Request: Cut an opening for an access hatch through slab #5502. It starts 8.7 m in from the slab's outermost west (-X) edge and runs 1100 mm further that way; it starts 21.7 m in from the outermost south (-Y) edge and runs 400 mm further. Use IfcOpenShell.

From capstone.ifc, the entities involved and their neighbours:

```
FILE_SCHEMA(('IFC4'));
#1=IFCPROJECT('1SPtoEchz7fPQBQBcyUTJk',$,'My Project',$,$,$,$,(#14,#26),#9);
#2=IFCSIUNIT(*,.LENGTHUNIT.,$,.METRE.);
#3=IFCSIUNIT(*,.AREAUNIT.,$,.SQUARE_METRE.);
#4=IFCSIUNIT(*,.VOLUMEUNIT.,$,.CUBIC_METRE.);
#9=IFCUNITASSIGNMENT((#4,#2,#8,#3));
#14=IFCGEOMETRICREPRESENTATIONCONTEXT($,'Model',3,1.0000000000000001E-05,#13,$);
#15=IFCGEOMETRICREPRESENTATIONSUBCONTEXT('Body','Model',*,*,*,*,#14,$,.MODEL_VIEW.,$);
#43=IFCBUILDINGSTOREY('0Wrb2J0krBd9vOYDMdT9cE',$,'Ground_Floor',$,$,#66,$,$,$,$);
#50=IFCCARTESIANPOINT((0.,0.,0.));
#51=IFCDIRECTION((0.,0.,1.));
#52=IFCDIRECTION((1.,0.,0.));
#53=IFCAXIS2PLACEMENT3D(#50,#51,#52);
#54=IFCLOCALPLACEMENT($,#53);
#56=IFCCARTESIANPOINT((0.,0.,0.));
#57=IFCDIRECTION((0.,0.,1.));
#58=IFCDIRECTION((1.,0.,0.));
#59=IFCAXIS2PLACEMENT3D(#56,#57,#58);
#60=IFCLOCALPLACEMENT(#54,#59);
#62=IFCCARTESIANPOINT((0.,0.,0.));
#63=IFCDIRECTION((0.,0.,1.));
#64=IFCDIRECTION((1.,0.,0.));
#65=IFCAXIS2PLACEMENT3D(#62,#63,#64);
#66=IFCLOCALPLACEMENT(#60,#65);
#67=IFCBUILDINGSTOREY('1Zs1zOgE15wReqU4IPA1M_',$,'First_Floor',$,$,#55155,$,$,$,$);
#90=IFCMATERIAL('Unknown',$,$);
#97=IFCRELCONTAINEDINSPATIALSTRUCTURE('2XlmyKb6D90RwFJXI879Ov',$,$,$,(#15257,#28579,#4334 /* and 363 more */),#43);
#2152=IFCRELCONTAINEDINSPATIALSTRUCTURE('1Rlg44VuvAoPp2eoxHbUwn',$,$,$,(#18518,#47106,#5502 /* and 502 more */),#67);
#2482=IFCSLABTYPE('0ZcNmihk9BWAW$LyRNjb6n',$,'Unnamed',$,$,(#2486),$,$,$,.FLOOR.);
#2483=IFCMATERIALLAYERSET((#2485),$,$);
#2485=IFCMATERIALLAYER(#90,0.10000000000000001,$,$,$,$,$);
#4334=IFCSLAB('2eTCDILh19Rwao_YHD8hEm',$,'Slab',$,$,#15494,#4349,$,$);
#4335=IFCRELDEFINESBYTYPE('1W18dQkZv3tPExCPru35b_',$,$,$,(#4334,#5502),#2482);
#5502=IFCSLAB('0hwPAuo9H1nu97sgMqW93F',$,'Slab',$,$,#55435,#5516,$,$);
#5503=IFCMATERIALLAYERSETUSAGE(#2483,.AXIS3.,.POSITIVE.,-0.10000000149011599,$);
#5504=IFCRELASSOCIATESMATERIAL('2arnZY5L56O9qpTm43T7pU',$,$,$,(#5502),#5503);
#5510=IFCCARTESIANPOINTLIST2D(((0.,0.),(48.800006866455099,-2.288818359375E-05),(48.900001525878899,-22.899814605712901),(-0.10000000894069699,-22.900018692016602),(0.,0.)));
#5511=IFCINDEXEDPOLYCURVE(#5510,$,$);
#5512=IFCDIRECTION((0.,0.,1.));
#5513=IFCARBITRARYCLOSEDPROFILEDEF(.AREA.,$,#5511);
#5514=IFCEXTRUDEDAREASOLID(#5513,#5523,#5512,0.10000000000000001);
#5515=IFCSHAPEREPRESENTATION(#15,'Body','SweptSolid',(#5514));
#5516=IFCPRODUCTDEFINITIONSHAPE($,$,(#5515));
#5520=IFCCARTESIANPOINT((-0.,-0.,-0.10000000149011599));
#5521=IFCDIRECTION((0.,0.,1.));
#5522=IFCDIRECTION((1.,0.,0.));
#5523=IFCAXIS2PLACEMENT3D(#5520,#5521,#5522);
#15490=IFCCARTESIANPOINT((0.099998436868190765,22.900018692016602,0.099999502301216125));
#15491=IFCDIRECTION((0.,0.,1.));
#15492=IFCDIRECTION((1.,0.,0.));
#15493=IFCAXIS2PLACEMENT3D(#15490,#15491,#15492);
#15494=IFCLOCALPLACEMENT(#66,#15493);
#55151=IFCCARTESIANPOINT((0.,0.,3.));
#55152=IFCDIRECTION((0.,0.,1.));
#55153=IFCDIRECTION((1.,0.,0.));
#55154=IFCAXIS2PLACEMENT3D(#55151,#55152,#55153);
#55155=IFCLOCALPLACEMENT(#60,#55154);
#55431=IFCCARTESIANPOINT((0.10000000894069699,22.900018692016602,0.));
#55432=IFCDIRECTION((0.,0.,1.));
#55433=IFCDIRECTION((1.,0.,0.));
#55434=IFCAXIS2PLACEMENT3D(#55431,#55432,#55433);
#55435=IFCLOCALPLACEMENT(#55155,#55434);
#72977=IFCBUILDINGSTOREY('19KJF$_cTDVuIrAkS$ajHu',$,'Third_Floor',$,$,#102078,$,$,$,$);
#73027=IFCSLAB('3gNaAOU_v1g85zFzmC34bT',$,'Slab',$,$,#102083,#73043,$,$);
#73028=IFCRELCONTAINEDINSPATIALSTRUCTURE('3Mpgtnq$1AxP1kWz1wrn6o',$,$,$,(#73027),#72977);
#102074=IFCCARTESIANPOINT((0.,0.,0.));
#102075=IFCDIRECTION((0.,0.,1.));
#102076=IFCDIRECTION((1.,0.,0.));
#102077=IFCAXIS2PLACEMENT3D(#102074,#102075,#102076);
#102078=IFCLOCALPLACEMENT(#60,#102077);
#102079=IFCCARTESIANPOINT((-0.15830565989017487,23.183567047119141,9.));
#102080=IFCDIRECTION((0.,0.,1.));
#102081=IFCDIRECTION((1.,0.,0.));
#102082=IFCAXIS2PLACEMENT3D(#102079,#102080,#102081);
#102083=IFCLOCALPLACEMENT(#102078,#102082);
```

```python
import numpy as np
import ifcopenshell
import ifcopenshell.api.feature
import ifcopenshell.api.geometry
import ifcopenshell.api.root
import ifcopenshell.geom
import ifcopenshell.util.placement
import ifcopenshell.util.representation
import ifcopenshell.util.shape
import ifcopenshell.util.unit

model = ifcopenshell.open("capstone.ifc")
unit_scale = ifcopenshell.util.unit.calculate_unit_scale(model)
settings = ifcopenshell.geom.settings()


def volume(element):
    """Net volume in cubic metres, openings subtracted."""
    shape = ifcopenshell.geom.create_shape(settings, element)
    return ifcopenshell.util.shape.get_volume(shape.geometry)


slab = model.by_guid("0hwPAuo9H1nu97sgMqW93F")
before = volume(slab)

# Extent in the slab's own axes, in metres. The edges named are its -X and -Y sides.
slab_shape = ifcopenshell.geom.create_shape(settings, slab)
vertices = ifcopenshell.util.shape.get_vertices(slab_shape.geometry)
x_min, y_min, bottom = vertices.min(axis=0)
top = vertices[:, 2].max()

opening = ifcopenshell.api.root.create_entity(model, ifc_class="IfcOpeningElement", name="Access hatch opening", predefined_type="OPENING")
context = ifcopenshell.util.representation.get_context(model, "Model", "Body", "MODEL_VIEW")
width, depth = 1.1, 0.4
outline = [(0.0, 0.0), (width, 0.0), (width, depth), (0.0, depth), (0.0, 0.0)]
# Overshoot both faces by 50 mm so the cut is clean.
shape = ifcopenshell.api.geometry.add_slab_representation(
    model, context=context, depth=top - bottom + 0.1, polyline=outline
)
ifcopenshell.api.geometry.assign_representation(model, product=opening, representation=shape)

matrix = ifcopenshell.util.placement.get_local_placement(slab.ObjectPlacement)
matrix[:, 3] = matrix @ np.append(np.array([x_min + 8.7, y_min + 21.7, bottom - 0.05]) / unit_scale, 1.0)
ifcopenshell.api.geometry.edit_object_placement(model, product=opening, matrix=matrix, is_si=False)
ifcopenshell.api.feature.add_feature(model, feature=opening, element=slab)

after = volume(slab)

print(f"slab volume {before:.3f} -> {after:.3f} m3")

model.write("capstone_edited.ifc")
```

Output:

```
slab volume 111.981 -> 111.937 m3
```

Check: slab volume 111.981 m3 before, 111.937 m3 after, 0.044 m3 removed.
